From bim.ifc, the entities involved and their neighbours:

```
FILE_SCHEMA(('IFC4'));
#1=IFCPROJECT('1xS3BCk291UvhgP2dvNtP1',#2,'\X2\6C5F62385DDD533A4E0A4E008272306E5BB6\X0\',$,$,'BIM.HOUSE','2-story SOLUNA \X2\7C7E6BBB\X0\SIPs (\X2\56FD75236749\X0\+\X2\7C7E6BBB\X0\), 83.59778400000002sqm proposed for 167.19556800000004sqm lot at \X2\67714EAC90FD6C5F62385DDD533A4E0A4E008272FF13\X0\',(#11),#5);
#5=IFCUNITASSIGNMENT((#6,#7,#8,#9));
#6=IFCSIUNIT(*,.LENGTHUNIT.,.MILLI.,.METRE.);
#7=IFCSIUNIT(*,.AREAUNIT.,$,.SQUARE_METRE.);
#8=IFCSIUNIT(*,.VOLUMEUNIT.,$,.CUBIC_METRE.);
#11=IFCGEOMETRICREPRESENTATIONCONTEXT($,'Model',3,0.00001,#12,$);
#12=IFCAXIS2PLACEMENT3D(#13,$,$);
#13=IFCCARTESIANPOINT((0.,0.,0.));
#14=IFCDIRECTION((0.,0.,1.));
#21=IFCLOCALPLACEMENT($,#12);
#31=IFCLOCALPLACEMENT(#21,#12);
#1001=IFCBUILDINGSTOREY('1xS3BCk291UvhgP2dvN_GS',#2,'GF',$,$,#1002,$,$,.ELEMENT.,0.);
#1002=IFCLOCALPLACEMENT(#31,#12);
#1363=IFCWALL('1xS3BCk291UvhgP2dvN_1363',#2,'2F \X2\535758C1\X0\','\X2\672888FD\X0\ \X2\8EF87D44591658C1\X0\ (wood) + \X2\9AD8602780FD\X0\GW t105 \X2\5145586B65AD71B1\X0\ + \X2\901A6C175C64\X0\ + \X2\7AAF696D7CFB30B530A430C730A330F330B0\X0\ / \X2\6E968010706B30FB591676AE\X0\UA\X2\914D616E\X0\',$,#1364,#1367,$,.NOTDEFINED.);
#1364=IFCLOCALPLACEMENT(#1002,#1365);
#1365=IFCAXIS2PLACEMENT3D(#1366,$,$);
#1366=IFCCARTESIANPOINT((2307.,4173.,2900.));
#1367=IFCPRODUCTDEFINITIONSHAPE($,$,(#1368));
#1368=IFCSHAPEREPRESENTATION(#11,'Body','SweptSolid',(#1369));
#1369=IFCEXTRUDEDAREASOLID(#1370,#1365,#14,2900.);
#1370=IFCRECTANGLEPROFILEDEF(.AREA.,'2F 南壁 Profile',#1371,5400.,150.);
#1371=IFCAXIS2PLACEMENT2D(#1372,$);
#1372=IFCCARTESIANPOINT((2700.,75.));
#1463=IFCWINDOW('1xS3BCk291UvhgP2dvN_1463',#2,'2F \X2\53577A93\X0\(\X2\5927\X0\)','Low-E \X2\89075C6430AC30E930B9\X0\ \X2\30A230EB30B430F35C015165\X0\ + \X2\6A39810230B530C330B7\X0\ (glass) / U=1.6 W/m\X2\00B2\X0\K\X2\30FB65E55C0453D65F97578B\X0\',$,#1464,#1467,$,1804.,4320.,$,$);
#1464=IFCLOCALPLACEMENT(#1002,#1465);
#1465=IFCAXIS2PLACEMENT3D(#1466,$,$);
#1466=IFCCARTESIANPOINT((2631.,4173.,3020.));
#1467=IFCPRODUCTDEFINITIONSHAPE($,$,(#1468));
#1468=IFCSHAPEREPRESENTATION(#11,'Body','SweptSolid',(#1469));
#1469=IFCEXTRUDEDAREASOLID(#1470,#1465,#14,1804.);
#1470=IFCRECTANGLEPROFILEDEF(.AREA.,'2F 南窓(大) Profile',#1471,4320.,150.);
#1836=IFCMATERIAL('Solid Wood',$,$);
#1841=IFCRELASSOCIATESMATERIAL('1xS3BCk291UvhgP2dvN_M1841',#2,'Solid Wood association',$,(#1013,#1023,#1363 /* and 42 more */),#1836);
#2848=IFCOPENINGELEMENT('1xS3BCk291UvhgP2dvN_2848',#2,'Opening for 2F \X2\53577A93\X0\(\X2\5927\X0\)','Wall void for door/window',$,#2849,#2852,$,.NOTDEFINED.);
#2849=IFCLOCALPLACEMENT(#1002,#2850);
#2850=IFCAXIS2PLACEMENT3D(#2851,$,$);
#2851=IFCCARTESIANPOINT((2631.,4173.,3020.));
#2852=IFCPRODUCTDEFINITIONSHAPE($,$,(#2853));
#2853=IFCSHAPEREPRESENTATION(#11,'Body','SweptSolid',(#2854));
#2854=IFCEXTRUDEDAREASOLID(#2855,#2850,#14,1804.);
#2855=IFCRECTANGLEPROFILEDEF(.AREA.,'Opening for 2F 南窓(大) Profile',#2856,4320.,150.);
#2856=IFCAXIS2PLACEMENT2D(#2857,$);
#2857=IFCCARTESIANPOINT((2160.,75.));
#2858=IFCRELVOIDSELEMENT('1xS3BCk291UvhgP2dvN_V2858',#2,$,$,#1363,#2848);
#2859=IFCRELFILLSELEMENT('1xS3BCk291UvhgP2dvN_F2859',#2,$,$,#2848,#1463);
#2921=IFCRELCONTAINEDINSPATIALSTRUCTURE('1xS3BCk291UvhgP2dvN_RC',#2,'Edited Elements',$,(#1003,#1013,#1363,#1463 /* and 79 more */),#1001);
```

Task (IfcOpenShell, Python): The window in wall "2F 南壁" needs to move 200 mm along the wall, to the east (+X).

```python
import ifcopenshell
import ifcopenshell.api.geometry
import ifcopenshell.util.placement
import ifcopenshell.util.unit

model = ifcopenshell.open("bim.ifc")
unit_scale = ifcopenshell.util.unit.calculate_unit_scale(model)

window = model.by_guid("1xS3BCk291UvhgP2dvN_1463")
opening = window.FillsVoids[0].RelatingOpeningElement
wall = opening.VoidsElements[0].RelatingBuildingElement

wall_matrix = ifcopenshell.util.placement.get_local_placement(wall.ObjectPlacement)
shift = wall_matrix[:3, 0] * 0.2 / unit_scale
before = ifcopenshell.util.placement.get_local_placement(window.ObjectPlacement)[:3, 3].copy()

# The window is not placed relative to its opening, so move both.
for product in (opening, window):
    matrix = ifcopenshell.util.placement.get_local_placement(product.ObjectPlacement)
    matrix[:3, 3] += shift
    ifcopenshell.api.geometry.edit_object_placement(model, product=product, matrix=matrix, is_si=False)

after = ifcopenshell.util.placement.get_local_placement(window.ObjectPlacement)[:3, 3]
print("window moved by", (after - before).round(3) + 0.0)

model.write("bim_updated.ifc")
```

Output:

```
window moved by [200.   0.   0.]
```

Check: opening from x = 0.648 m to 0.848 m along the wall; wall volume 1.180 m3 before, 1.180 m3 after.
